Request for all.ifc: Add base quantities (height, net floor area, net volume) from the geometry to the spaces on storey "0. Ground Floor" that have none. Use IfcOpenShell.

First a look at what the model holds.

```python
import ifcopenshell
import ifcopenshell.util.element
import ifcopenshell.util.unit

model = ifcopenshell.open("all.ifc")
print(model.schema)
for unit_type in ("LENGTHUNIT", "AREAUNIT", "VOLUMEUNIT"):
    print(unit_type, ifcopenshell.util.unit.calculate_unit_scale(model, unit_type))
storey = next(s for s in model.by_type("IfcBuildingStorey") if s.Name == "0. Ground Floor")
spaces = [e for e in ifcopenshell.util.element.get_decomposition(storey) if e.is_a("IfcSpace")]
for e in sorted(spaces, key=lambda e: e.id()):
    print(e.id(), e.is_a(), e.Name, list(ifcopenshell.util.element.get_psets(e, qtos_only=True)), sep=" | ")
```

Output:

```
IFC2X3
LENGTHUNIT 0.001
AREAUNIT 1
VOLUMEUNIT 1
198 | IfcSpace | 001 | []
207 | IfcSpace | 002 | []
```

```python
import ifcopenshell
import ifcopenshell.api.pset
import ifcopenshell.geom
import ifcopenshell.util.element
import ifcopenshell.util.shape
import ifcopenshell.util.unit

model = ifcopenshell.open("all.ifc")
unit_scale = ifcopenshell.util.unit.calculate_unit_scale(model)
area_scale = ifcopenshell.util.unit.calculate_unit_scale(model, "AREAUNIT")
volume_scale = ifcopenshell.util.unit.calculate_unit_scale(model, "VOLUMEUNIT")
settings = ifcopenshell.geom.settings()

storey = next(s for s in model.by_type("IfcBuildingStorey") if s.Name == "0. Ground Floor")
spaces = [e for e in ifcopenshell.util.element.get_decomposition(storey) if e.is_a("IfcSpace")]

for e in sorted(spaces, key=lambda e: e.id()):
    if ifcopenshell.util.element.get_psets(e, qtos_only=True, should_inherit=False):
        continue
    # Geometry comes back in metres, in the element's own axes.
    shape = ifcopenshell.geom.create_shape(settings, e)
    values = {
        "Height": ifcopenshell.util.shape.get_z(shape.geometry) / unit_scale,
        "NetFloorArea": ifcopenshell.util.shape.get_footprint_area(shape.geometry) / area_scale,
        "NetVolume": ifcopenshell.util.shape.get_volume(shape.geometry) / volume_scale,
    }
    qto = ifcopenshell.api.pset.add_qto(model, product=e, name="BaseQuantities")
    ifcopenshell.api.pset.edit_qto(model, qto=qto, properties=values)
    print(e.id(), {k: round(v, 3) for k, v in values.items()})

model.write("all_rev.ifc")
```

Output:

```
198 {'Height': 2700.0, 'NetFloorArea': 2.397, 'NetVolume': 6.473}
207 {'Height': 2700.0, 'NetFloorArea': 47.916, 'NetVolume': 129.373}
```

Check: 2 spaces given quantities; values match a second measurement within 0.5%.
